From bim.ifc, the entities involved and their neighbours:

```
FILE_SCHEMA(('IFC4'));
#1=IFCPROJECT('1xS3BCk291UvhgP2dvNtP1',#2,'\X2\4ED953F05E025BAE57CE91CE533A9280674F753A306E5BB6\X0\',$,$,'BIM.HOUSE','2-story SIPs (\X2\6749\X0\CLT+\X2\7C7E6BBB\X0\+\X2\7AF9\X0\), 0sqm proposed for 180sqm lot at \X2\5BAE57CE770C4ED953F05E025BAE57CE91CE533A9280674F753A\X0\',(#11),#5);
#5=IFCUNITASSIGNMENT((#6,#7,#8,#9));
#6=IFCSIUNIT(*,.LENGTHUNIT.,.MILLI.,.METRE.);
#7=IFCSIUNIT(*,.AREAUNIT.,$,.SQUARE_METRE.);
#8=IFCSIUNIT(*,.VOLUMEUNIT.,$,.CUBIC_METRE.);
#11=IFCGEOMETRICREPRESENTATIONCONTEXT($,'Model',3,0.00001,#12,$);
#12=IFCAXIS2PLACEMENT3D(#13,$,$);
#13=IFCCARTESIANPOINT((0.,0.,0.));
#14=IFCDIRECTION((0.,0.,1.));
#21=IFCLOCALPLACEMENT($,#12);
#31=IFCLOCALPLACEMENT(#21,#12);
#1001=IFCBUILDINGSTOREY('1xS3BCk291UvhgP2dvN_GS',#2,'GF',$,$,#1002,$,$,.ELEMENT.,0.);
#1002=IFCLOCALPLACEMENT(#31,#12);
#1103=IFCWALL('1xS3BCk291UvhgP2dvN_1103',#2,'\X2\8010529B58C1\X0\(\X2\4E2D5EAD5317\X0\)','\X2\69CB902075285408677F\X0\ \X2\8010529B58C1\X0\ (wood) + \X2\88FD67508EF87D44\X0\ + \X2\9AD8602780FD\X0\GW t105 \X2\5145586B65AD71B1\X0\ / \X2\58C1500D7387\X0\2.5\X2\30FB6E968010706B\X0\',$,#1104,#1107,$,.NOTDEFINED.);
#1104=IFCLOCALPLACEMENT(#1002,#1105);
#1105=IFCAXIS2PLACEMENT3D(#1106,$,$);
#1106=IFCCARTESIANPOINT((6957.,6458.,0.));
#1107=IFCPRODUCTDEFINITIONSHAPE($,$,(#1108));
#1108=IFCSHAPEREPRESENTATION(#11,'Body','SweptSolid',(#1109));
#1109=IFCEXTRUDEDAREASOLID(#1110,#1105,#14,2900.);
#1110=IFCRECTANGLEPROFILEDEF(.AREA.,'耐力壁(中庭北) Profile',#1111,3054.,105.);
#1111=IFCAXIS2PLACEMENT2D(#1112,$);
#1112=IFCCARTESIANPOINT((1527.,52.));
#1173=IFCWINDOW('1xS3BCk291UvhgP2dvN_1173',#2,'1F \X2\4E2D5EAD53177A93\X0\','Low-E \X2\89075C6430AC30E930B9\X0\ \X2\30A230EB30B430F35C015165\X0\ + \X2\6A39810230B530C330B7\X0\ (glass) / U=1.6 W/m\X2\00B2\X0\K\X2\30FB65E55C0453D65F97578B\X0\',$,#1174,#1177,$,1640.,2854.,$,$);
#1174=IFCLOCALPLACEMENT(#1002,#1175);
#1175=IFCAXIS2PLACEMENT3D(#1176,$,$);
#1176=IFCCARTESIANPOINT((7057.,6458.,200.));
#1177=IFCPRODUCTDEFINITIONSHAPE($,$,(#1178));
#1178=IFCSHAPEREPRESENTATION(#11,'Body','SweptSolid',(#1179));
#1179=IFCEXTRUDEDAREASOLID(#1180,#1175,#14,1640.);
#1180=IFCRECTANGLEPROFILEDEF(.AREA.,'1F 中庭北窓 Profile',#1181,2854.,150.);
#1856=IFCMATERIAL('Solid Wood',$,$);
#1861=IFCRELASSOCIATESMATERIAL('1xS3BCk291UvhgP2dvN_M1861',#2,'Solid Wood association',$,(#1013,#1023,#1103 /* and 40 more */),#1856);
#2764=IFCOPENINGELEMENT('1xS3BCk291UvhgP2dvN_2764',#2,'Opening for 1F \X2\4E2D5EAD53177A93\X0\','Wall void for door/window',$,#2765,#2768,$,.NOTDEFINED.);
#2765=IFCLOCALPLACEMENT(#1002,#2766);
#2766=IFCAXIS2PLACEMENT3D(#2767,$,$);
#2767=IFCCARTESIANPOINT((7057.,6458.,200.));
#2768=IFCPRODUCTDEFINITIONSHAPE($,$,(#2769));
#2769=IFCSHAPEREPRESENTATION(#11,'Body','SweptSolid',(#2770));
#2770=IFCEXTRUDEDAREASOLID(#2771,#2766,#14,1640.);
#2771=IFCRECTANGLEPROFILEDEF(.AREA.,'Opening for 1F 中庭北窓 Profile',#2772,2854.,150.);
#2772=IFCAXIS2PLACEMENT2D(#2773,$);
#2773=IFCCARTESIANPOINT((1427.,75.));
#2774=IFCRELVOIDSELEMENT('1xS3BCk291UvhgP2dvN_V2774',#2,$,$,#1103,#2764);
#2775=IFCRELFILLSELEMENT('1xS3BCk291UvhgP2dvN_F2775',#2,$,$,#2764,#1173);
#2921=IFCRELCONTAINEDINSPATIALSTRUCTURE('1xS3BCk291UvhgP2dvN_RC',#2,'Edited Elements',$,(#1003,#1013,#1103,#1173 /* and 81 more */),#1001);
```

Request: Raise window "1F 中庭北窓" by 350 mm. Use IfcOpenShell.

```python
import numpy as np
import ifcopenshell
import ifcopenshell.api.geometry
import ifcopenshell.util.placement
import ifcopenshell.util.unit

model = ifcopenshell.open("bim.ifc")
unit_scale = ifcopenshell.util.unit.calculate_unit_scale(model)

window = model.by_id(1173)
opening = window.FillsVoids[0].RelatingOpeningElement
dz = 0.35 / unit_scale

shift = np.array([0.0, 0.0, dz])
# The window is not placed relative to its opening, so move both.
for product in (opening, window):
    matrix = ifcopenshell.util.placement.get_local_placement(product.ObjectPlacement)
    matrix[:3, 3] += shift
    ifcopenshell.api.geometry.edit_object_placement(model, product=product, matrix=matrix, is_si=False)

print(f"moved by {dz * unit_scale:+.3f} m")

model.write("bim_edited.ifc")
```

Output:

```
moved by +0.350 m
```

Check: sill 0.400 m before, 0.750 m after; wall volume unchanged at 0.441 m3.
